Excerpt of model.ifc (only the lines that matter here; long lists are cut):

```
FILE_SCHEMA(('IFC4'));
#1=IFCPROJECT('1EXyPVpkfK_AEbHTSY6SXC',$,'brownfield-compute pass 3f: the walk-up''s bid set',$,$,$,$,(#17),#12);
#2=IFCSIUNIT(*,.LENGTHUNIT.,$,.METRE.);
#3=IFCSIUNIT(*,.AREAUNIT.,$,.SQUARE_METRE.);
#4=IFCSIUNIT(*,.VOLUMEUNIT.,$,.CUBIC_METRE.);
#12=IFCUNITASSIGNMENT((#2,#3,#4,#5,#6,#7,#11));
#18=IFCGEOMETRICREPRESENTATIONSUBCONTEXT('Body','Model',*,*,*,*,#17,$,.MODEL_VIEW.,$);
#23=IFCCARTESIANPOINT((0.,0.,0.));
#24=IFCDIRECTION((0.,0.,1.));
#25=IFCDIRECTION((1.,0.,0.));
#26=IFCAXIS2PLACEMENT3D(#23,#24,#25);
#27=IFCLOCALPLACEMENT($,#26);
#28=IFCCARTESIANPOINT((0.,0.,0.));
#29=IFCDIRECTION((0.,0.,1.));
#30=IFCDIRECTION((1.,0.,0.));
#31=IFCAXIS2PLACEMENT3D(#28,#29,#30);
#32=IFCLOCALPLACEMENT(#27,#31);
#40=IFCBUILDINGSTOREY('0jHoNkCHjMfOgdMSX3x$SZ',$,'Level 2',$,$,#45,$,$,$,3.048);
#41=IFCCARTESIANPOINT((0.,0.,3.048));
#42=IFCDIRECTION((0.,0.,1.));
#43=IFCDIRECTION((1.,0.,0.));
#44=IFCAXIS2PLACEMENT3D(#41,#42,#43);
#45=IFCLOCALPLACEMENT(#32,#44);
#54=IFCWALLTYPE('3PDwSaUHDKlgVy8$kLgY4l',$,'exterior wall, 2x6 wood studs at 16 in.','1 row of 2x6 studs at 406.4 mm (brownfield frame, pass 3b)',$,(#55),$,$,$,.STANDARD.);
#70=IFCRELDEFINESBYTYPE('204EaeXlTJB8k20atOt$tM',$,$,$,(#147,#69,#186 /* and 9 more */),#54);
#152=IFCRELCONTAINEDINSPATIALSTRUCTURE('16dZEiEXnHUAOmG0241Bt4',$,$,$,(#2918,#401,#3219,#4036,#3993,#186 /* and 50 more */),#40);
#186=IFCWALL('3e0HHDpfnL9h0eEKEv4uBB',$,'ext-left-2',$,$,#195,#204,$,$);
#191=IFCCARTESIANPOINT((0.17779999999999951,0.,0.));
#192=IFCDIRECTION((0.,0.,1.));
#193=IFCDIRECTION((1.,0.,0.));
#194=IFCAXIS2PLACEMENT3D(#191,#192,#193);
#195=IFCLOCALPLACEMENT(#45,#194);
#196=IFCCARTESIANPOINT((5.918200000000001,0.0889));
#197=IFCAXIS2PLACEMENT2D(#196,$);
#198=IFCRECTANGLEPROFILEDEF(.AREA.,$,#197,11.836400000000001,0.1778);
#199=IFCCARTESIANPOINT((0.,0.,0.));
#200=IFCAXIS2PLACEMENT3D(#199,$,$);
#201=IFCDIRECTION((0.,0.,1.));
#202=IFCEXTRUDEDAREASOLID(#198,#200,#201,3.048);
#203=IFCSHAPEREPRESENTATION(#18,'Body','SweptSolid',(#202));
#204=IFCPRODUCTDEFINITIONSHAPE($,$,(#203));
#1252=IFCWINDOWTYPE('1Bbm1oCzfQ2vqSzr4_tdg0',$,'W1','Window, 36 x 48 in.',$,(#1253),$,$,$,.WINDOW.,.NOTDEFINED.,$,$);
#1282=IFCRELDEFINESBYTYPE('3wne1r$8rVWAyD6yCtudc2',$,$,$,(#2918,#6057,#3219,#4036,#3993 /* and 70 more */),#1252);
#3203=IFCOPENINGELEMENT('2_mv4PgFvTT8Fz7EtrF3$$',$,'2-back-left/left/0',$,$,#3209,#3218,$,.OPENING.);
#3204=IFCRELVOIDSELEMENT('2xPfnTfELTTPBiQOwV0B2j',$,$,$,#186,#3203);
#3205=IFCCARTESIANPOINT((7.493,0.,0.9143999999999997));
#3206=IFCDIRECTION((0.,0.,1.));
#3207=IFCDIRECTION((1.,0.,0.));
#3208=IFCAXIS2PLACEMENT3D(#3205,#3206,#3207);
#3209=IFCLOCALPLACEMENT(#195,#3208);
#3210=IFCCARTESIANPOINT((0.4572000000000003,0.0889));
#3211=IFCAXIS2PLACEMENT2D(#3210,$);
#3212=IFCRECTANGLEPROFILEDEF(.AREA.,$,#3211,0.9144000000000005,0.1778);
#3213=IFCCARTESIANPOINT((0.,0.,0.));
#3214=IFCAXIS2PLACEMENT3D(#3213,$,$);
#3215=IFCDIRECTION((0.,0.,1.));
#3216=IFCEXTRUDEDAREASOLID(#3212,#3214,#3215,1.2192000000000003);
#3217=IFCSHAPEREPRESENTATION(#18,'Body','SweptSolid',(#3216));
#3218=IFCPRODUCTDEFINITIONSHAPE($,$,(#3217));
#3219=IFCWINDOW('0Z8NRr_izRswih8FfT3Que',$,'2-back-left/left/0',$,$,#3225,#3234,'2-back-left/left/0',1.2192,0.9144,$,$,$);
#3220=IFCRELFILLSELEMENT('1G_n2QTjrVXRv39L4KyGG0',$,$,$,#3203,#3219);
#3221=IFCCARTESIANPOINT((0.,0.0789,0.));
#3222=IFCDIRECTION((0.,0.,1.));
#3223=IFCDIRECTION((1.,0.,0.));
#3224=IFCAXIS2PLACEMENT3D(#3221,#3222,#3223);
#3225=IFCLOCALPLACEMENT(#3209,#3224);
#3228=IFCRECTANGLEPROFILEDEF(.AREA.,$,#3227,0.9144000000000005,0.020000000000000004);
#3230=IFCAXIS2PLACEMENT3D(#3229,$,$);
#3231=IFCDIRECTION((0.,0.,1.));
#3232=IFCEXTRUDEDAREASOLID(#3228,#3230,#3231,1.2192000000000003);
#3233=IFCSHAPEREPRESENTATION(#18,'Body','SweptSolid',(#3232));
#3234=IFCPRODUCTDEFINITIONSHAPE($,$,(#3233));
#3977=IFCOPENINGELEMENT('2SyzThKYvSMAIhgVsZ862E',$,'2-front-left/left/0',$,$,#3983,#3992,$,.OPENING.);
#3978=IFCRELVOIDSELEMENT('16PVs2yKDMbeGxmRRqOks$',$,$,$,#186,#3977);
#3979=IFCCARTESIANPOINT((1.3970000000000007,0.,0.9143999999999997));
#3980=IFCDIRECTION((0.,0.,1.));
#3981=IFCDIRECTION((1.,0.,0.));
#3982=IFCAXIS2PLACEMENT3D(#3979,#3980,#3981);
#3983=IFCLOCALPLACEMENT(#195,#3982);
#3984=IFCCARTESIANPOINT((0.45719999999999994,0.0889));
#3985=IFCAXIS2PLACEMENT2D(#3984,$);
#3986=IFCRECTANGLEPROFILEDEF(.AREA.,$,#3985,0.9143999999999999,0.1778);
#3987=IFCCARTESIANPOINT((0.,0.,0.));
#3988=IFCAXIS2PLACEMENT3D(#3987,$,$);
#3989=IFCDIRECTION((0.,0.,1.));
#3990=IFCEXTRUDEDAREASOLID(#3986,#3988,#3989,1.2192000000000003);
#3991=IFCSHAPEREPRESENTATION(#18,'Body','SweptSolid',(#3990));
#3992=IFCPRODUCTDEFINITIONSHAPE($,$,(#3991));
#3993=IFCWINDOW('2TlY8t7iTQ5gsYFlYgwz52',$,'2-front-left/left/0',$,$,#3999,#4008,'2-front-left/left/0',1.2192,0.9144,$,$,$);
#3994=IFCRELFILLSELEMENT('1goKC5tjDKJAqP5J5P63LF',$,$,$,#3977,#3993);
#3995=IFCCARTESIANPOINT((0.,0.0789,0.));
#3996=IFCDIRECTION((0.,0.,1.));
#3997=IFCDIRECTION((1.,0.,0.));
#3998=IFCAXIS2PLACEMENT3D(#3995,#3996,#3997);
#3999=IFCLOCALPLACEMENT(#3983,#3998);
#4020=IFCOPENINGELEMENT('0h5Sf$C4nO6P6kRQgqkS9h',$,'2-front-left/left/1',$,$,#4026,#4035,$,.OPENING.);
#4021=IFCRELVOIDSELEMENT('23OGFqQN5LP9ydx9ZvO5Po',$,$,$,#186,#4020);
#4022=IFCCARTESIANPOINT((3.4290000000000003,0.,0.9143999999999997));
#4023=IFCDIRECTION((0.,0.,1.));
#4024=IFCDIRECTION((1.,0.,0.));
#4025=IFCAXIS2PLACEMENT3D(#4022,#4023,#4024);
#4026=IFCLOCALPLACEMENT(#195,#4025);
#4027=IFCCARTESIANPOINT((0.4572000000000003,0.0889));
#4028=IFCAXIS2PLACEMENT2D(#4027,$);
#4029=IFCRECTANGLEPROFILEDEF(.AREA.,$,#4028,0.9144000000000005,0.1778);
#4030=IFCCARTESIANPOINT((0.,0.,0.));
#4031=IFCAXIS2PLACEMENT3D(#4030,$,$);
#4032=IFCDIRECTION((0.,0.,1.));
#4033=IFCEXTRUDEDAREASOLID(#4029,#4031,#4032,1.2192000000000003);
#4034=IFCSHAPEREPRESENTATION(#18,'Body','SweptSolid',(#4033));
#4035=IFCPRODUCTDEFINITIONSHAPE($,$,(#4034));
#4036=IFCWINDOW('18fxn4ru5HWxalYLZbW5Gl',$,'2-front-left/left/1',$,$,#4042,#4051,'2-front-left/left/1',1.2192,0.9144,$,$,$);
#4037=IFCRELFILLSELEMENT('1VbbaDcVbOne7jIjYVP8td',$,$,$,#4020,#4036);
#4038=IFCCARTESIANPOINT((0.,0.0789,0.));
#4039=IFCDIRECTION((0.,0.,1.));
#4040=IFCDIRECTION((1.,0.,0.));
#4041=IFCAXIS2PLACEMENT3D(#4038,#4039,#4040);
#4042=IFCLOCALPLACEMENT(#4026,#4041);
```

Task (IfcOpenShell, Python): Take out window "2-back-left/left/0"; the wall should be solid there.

```python
import ifcopenshell
import ifcopenshell.api.feature
import ifcopenshell.api.root
import ifcopenshell.geom
import ifcopenshell.util.shape

model = ifcopenshell.open("model.ifc")
settings = ifcopenshell.geom.settings()


def volume(element):
    """Net volume in cubic metres, openings subtracted."""
    shape = ifcopenshell.geom.create_shape(settings, element)
    return ifcopenshell.util.shape.get_volume(shape.geometry)


window = model.by_id(3219)
opening = window.FillsVoids[0].RelatingOpeningElement
wall = opening.VoidsElements[0].RelatingBuildingElement
before = volume(wall)

ifcopenshell.api.root.remove_product(model, product=window)
ifcopenshell.api.feature.remove_feature(model, feature=opening)

after = volume(wall)

print(f"wall volume {before:.3f} -> {after:.3f} m3")

model.write("model_v2.ifc")
```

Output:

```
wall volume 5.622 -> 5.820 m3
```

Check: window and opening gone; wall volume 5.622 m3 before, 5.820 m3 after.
